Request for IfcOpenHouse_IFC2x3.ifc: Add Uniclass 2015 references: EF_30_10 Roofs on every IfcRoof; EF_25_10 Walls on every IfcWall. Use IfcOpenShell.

First a look at what the model holds.

```python
import ifcopenshell

model = ifcopenshell.open("IfcOpenHouse_IFC2x3.ifc")
print(model.schema)
print("classifications:", [c.Name for c in model.by_type("IfcClassification")])
for ifc_class in ("IfcDoor", "IfcRoof", "IfcStair", "IfcWall", "IfcWindow"):
    print(ifc_class, len(model.by_type(ifc_class)))
```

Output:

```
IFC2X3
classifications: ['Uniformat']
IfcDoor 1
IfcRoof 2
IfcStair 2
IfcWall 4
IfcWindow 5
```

```python
import ifcopenshell
import ifcopenshell.api.classification

model = ifcopenshell.open("IfcOpenHouse_IFC2x3.ifc")

# IFC2X3 requires Source and Edition and has no link from the project to the system.
system = model.create_entity("IfcClassification", Source="NBS", Edition="2015", Name="Uniclass 2015")

codes = {
    "IfcRoof": ("EF_30_10", "Roofs"),
    "IfcWall": ("EF_25_10", "Walls"),
}
for ifc_class, (code, name) in codes.items():
    products = model.by_type(ifc_class)
    ifcopenshell.api.classification.add_reference(
        model, products=products, classification=system, identification=code, name=name
    )
    print(code, len(products))

model.write("IfcOpenHouse_IFC2x3-out.ifc")
```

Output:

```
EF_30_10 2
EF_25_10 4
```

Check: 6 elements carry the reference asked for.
